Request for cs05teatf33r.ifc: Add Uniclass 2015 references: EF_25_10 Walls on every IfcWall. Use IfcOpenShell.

First a look at what the model holds.

```python
import ifcopenshell

model = ifcopenshell.open("cs05teatf33r.ifc")
print(model.schema)
print("classifications:", [c.Name for c in model.by_type("IfcClassification")])
for ifc_class in ("IfcDoor", "IfcRoof", "IfcStair", "IfcWall", "IfcWindow"):
    print(ifc_class, len(model.by_type(ifc_class)))
```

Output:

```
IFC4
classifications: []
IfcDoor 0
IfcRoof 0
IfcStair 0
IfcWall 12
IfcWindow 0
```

```python
import ifcopenshell
import ifcopenshell.api.classification

model = ifcopenshell.open("cs05teatf33r.ifc")

system = ifcopenshell.api.classification.add_classification(model, classification="Uniclass 2015")

codes = {
    "IfcWall": ("EF_25_10", "Walls"),
}
for ifc_class, (code, name) in codes.items():
    products = model.by_type(ifc_class)
    ifcopenshell.api.classification.add_reference(
        model, products=products, classification=system, identification=code, name=name
    )
    print(code, len(products))

model.write("cs05teatf33r_updated.ifc")
```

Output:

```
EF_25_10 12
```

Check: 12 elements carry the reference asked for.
